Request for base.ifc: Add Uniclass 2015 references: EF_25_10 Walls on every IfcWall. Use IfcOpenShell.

First a look at what the model holds.

```python
import ifcopenshell

model = ifcopenshell.open("base.ifc")
print(model.schema)
print("classifications:", [c.Name for c in model.by_type("IfcClassification")])
for ifc_class in ("IfcDoor", "IfcRoof", "IfcStair", "IfcWall", "IfcWindow"):
    print(ifc_class, len(model.by_type(ifc_class)))
```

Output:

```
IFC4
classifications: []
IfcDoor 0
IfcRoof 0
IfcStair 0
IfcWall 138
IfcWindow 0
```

```python
import ifcopenshell
import ifcopenshell.api.classification

model = ifcopenshell.open("base.ifc")

system = ifcopenshell.api.classification.add_classification(model, classification="Uniclass 2015")

codes = {
    "IfcWall": ("EF_25_10", "Walls"),
}
for ifc_class, (code, name) in codes.items():
    products = model.by_type(ifc_class)
    ifcopenshell.api.classification.add_reference(
        model, products=products, classification=system, identification=code, name=name
    )
    print(code, len(products))

model.write("base_updated.ifc")
```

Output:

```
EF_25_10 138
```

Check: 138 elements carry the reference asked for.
